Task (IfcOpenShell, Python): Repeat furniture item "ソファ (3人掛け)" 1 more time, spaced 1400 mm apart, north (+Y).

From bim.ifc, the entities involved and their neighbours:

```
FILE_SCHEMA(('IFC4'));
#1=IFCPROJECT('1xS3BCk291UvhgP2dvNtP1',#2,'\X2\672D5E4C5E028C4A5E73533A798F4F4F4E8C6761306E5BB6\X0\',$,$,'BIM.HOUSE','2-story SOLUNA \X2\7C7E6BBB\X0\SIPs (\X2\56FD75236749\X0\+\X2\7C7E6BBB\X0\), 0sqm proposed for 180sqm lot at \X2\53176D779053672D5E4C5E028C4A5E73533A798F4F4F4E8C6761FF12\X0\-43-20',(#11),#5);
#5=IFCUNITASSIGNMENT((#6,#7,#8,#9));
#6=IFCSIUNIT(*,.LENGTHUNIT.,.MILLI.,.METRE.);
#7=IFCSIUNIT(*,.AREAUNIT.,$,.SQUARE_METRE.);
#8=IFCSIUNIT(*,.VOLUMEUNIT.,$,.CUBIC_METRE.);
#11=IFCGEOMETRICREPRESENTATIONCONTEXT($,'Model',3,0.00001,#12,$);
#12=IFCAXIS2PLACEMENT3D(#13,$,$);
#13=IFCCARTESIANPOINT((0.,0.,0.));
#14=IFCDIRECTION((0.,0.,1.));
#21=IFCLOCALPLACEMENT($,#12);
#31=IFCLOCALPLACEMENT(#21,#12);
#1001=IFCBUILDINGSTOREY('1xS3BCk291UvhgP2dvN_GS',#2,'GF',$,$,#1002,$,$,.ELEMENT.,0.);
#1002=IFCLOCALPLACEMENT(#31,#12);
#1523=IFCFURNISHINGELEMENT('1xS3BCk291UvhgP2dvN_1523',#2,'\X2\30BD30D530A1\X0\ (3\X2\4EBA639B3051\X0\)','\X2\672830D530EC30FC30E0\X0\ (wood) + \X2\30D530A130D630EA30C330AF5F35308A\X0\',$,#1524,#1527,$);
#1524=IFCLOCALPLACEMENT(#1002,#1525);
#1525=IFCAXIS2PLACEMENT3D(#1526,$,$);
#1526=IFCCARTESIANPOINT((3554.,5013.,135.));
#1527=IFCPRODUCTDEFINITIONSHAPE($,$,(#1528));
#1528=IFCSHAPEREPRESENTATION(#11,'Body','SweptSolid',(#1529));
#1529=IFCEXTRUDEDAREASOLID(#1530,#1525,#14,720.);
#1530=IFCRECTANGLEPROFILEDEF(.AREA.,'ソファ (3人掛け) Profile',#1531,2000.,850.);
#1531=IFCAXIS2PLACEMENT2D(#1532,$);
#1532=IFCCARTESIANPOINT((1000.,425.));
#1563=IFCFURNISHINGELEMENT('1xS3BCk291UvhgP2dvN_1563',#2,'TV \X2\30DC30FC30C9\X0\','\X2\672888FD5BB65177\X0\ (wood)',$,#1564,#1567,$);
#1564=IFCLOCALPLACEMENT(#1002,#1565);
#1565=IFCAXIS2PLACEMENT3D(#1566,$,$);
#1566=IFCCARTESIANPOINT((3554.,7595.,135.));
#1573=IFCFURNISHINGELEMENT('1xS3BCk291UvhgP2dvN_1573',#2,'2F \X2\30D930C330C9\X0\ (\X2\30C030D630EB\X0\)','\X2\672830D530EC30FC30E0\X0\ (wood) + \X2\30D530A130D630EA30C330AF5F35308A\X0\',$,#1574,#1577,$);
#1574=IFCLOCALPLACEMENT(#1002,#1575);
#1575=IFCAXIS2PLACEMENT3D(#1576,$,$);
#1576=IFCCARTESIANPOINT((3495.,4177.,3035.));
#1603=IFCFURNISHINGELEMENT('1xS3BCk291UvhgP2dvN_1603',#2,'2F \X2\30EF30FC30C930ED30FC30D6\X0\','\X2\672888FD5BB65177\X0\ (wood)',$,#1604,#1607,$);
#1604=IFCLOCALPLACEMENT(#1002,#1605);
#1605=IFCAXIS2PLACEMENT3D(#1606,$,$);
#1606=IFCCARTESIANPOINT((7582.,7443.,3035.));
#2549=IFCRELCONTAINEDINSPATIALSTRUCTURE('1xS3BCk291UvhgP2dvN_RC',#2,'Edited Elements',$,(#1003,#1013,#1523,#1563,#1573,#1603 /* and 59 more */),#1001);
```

```python
import numpy as np
import ifcopenshell
import ifcopenshell.api.geometry
import ifcopenshell.api.root
import ifcopenshell.util.element
import ifcopenshell.util.placement

model = ifcopenshell.open("bim.ifc")


def reuse_history(source, copy):
    """copy_class also copies each property set's owner history, people and application; keep the originals."""
    for rel in copy.IsDefinedBy:
        if rel.is_a("IfcRelDefinesByProperties") and (history := rel.RelatingPropertyDefinition.OwnerHistory):
            rel.RelatingPropertyDefinition.OwnerHistory = source.OwnerHistory
            ifcopenshell.util.element.remove_deep2(model, history)


source = model.by_guid("1xS3BCk291UvhgP2dvN_1523")
base = ifcopenshell.util.placement.get_local_placement(source.ObjectPlacement)
step = np.array([0.0, 1.0, 0.0]) * 1400.0

for i in range(1, 2):
    copy = ifcopenshell.api.root.copy_class(model, product=source)
    copy.Representation = ifcopenshell.util.element.copy_deep(
        model, source.Representation, exclude=["IfcGeometricRepresentationContext", "IfcRepresentationMap"]
    )
    reuse_history(source, copy)
    matrix = base.copy()
    matrix[:3, 3] += i * step
    print("added at", matrix[:3, 3].round(3) + 0.0)
    ifcopenshell.api.geometry.edit_object_placement(model, product=copy, matrix=matrix, is_si=False)

model.write("bim_edited.ifc")
```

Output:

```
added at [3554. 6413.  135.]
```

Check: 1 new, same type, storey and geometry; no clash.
